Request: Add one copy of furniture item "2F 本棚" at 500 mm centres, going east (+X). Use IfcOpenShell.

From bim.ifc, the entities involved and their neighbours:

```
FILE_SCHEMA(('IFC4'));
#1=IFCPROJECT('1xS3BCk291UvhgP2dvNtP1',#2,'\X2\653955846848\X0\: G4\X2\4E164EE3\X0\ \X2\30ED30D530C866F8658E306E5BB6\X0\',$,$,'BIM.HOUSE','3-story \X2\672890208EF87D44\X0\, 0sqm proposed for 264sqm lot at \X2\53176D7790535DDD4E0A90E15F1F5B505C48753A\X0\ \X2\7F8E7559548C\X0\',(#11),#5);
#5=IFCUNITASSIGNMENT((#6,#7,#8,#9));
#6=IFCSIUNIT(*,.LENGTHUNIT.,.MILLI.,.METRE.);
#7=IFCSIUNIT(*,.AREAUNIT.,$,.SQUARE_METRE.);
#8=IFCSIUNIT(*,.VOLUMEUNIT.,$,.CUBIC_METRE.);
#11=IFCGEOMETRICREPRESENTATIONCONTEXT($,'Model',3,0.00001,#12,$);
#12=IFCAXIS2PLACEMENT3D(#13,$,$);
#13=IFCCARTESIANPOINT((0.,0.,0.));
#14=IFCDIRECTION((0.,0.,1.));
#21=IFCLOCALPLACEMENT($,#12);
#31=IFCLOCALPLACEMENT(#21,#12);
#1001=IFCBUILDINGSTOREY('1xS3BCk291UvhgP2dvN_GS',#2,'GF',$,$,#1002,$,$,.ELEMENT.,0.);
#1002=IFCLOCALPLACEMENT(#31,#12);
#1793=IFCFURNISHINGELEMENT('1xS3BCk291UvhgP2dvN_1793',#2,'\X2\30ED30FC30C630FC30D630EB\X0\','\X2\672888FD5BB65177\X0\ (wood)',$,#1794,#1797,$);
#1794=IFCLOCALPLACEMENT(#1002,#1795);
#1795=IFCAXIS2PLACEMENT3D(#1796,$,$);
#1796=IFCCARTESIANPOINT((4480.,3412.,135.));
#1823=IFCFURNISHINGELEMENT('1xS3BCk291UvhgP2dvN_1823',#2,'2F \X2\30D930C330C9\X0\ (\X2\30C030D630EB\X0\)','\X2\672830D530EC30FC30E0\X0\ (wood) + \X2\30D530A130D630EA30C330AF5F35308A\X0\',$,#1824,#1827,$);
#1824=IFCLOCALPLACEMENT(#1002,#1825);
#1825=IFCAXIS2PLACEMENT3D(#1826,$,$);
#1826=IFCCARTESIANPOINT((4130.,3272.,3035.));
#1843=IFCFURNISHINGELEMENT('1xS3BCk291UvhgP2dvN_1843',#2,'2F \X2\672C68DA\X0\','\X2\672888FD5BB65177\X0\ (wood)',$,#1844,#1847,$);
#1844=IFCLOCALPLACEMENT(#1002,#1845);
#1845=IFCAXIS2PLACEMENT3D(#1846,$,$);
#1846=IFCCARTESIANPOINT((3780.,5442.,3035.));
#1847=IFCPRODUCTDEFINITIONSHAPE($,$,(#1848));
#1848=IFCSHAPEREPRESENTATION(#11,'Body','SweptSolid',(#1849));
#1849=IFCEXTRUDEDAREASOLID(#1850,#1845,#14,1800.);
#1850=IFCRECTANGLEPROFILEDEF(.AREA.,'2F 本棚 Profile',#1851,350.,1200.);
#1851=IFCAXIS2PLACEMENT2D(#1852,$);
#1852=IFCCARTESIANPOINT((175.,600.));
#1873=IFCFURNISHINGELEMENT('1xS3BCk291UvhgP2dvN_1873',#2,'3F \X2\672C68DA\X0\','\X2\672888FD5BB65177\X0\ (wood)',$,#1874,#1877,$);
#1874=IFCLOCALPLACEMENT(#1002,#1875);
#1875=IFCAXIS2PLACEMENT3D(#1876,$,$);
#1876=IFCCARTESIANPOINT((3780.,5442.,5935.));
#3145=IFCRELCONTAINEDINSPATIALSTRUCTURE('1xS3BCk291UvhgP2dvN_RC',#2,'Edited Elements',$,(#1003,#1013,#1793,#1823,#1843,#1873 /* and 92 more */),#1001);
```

```python
import numpy as np
import ifcopenshell
import ifcopenshell.api.geometry
import ifcopenshell.api.root
import ifcopenshell.util.element
import ifcopenshell.util.placement
import ifcopenshell.util.unit

model = ifcopenshell.open("bim.ifc")
unit_scale = ifcopenshell.util.unit.calculate_unit_scale(model)


def reuse_history(source, copy):
    """copy_class also copies each property set's owner history, people and application; keep the originals."""
    for rel in copy.IsDefinedBy:
        if rel.is_a("IfcRelDefinesByProperties") and (history := rel.RelatingPropertyDefinition.OwnerHistory):
            rel.RelatingPropertyDefinition.OwnerHistory = source.OwnerHistory
            ifcopenshell.util.element.remove_deep2(model, history)


source = model.by_guid("1xS3BCk291UvhgP2dvN_1843")
base = ifcopenshell.util.placement.get_local_placement(source.ObjectPlacement)
step = np.array([1.0, 0.0, 0.0]) * 0.5 / unit_scale

for i in range(1, 2):
    copy = ifcopenshell.api.root.copy_class(model, product=source)
    copy.Representation = ifcopenshell.util.element.copy_deep(
        model, source.Representation, exclude=["IfcGeometricRepresentationContext", "IfcRepresentationMap"]
    )
    reuse_history(source, copy)
    matrix = base.copy()
    matrix[:3, 3] += i * step
    print("added at", matrix[:3, 3].round(3) + 0.0)
    ifcopenshell.api.geometry.edit_object_placement(model, product=copy, matrix=matrix, is_si=False)

model.write("bim_v2.ifc")
```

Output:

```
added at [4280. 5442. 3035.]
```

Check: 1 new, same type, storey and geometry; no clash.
